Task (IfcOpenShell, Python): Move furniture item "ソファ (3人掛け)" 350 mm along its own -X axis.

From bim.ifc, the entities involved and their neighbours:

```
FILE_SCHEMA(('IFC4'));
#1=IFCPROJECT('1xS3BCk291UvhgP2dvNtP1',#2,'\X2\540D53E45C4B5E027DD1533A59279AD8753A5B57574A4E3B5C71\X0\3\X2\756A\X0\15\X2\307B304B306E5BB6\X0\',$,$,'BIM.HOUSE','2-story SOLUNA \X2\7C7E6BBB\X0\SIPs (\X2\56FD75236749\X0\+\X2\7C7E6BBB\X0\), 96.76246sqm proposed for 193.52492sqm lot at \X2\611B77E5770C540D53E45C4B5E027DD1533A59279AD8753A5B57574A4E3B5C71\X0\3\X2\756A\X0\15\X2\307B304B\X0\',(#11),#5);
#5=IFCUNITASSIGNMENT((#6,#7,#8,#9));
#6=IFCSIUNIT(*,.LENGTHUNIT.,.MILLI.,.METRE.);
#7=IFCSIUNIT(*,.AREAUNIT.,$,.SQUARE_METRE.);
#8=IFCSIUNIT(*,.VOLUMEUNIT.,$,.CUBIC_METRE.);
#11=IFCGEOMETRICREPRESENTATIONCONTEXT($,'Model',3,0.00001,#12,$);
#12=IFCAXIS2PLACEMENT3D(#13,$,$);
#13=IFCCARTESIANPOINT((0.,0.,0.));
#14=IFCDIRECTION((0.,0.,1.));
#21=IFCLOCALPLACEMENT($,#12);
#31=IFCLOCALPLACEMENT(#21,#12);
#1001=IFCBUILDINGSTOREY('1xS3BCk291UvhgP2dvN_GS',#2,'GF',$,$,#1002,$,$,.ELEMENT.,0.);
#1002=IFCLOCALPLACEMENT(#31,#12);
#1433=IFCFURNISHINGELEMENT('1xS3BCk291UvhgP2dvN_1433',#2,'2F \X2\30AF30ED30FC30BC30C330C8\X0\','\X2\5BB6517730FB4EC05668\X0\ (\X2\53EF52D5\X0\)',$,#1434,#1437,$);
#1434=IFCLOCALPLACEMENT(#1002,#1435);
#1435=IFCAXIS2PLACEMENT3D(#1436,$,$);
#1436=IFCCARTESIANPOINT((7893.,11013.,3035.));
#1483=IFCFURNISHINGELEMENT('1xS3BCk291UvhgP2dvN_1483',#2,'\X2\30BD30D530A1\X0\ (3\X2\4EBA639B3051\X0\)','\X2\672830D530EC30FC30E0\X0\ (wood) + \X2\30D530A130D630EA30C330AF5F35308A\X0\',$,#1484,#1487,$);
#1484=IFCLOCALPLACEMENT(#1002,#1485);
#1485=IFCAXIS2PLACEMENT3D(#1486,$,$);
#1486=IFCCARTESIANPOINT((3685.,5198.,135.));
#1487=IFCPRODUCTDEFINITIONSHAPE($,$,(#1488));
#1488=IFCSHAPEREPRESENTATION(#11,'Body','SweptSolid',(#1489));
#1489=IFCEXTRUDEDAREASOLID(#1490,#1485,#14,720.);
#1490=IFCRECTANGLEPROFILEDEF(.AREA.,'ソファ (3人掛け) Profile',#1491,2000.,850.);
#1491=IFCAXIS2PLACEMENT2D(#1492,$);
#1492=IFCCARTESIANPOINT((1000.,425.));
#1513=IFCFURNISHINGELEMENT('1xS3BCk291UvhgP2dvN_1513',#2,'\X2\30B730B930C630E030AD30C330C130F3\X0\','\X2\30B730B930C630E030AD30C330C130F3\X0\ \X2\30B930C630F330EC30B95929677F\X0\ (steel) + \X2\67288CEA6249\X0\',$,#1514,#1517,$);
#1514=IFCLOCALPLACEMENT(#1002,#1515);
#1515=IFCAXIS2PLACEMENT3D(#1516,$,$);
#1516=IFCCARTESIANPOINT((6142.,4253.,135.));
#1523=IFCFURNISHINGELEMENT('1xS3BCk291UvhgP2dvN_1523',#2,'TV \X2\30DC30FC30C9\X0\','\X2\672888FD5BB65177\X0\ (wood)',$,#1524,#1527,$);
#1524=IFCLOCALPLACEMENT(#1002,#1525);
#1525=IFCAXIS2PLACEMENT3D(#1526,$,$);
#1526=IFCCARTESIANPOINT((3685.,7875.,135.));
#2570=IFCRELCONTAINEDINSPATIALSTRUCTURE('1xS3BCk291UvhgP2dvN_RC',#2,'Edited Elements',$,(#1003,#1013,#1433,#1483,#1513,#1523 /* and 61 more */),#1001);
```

```python
import ifcopenshell
import ifcopenshell.api.geometry
import ifcopenshell.util.placement
import ifcopenshell.util.unit

model = ifcopenshell.open("bim.ifc")
unit_scale = ifcopenshell.util.unit.calculate_unit_scale(model)

item = model.by_guid("1xS3BCk291UvhgP2dvN_1483")
matrix = ifcopenshell.util.placement.get_local_placement(item.ObjectPlacement)
matrix[:3, 3] -= matrix[:3, 0] * 0.35 / unit_scale
ifcopenshell.api.geometry.edit_object_placement(model, product=item, matrix=matrix, is_si=False)

print(ifcopenshell.util.placement.get_local_placement(item.ObjectPlacement).round(3) + 0.0)

model.write("bim_edited.ifc")
```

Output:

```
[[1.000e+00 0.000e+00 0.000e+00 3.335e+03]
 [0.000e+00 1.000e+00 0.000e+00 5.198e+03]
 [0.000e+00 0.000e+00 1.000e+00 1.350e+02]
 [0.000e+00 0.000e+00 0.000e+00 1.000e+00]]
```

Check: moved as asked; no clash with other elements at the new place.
